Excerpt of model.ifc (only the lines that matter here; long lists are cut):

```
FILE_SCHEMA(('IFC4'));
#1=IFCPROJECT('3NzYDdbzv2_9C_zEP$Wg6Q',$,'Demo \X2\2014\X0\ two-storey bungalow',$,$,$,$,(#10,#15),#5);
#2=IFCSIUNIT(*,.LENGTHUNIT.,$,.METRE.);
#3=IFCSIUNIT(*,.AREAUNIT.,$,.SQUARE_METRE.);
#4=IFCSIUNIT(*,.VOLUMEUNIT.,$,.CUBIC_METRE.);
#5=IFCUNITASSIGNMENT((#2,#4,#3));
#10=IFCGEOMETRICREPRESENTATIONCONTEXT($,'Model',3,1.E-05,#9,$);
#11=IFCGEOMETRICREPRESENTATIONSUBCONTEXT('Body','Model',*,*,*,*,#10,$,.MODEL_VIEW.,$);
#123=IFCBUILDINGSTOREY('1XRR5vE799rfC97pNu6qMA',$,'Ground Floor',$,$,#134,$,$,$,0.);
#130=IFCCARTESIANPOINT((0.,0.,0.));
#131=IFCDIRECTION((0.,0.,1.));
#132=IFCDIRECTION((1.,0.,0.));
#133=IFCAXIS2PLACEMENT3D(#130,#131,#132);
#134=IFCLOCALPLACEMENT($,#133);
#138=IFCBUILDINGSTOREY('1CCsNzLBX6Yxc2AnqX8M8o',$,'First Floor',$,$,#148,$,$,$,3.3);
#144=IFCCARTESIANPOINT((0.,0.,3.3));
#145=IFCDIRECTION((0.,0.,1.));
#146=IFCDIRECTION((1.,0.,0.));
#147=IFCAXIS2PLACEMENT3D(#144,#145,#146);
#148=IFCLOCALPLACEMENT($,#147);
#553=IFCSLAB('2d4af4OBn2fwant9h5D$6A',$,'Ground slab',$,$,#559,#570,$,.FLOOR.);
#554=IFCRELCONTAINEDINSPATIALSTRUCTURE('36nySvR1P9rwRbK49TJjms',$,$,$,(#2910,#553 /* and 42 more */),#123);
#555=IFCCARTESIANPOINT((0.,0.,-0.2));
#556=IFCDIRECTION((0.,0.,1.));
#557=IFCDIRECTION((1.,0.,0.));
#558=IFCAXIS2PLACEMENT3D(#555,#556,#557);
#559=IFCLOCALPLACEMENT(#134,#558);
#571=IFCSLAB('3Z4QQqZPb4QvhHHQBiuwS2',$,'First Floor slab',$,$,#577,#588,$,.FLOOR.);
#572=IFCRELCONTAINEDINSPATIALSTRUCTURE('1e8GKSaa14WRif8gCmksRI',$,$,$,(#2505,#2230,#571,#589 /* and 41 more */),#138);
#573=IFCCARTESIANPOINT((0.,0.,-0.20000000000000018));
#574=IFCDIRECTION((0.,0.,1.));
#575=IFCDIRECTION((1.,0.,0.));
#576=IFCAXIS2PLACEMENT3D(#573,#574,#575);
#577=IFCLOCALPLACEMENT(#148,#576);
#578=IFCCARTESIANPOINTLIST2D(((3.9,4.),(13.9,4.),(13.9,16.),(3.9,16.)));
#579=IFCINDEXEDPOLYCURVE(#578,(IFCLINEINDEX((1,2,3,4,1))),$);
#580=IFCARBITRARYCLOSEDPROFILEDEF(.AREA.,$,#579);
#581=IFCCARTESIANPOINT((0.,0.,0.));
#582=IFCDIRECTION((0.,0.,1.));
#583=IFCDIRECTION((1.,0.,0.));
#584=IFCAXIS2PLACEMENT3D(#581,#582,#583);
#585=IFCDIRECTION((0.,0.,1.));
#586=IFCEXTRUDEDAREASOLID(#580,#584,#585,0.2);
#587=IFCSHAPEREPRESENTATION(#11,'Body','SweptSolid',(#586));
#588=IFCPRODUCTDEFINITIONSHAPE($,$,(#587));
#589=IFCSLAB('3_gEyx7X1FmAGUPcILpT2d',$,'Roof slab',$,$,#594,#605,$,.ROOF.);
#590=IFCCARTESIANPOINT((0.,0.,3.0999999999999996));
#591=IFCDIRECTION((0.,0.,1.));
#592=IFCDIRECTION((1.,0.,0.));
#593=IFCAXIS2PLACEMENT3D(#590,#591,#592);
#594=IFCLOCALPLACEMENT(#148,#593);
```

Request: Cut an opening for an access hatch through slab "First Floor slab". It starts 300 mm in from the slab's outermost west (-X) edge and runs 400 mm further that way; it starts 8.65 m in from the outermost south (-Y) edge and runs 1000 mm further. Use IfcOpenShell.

```python
import numpy as np
import ifcopenshell
import ifcopenshell.api.feature
import ifcopenshell.api.geometry
import ifcopenshell.api.root
import ifcopenshell.geom
import ifcopenshell.util.placement
import ifcopenshell.util.representation
import ifcopenshell.util.shape
import ifcopenshell.util.unit

model = ifcopenshell.open("model.ifc")
unit_scale = ifcopenshell.util.unit.calculate_unit_scale(model)
settings = ifcopenshell.geom.settings()


def volume(element):
    """Net volume in cubic metres, openings subtracted."""
    shape = ifcopenshell.geom.create_shape(settings, element)
    return ifcopenshell.util.shape.get_volume(shape.geometry)


slab = model.by_guid("3Z4QQqZPb4QvhHHQBiuwS2")
before = volume(slab)

# Extent in the slab's own axes, in metres. The edges named are its -X and -Y sides.
slab_shape = ifcopenshell.geom.create_shape(settings, slab)
vertices = ifcopenshell.util.shape.get_vertices(slab_shape.geometry)
x_min, y_min, bottom = vertices.min(axis=0)
top = vertices[:, 2].max()

opening = ifcopenshell.api.root.create_entity(model, ifc_class="IfcOpeningElement", name="Access hatch opening", predefined_type="OPENING")
context = ifcopenshell.util.representation.get_context(model, "Model", "Body", "MODEL_VIEW")
width, depth = 0.4, 1
outline = [(0.0, 0.0), (width, 0.0), (width, depth), (0.0, depth), (0.0, 0.0)]
# Overshoot both faces by 50 mm so the cut is clean.
shape = ifcopenshell.api.geometry.add_slab_representation(
    model, context=context, depth=top - bottom + 0.1, polyline=outline
)
ifcopenshell.api.geometry.assign_representation(model, product=opening, representation=shape)

matrix = ifcopenshell.util.placement.get_local_placement(slab.ObjectPlacement)
matrix[:, 3] = matrix @ np.append(np.array([x_min + 0.3, y_min + 8.65, bottom - 0.05]) / unit_scale, 1.0)
ifcopenshell.api.geometry.edit_object_placement(model, product=opening, matrix=matrix, is_si=False)
ifcopenshell.api.feature.add_feature(model, feature=opening, element=slab)

after = volume(slab)

print(f"slab volume {before:.3f} -> {after:.3f} m3")

model.write("model_edited.ifc")
```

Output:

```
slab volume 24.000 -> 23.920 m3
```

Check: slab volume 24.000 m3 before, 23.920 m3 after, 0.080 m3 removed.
